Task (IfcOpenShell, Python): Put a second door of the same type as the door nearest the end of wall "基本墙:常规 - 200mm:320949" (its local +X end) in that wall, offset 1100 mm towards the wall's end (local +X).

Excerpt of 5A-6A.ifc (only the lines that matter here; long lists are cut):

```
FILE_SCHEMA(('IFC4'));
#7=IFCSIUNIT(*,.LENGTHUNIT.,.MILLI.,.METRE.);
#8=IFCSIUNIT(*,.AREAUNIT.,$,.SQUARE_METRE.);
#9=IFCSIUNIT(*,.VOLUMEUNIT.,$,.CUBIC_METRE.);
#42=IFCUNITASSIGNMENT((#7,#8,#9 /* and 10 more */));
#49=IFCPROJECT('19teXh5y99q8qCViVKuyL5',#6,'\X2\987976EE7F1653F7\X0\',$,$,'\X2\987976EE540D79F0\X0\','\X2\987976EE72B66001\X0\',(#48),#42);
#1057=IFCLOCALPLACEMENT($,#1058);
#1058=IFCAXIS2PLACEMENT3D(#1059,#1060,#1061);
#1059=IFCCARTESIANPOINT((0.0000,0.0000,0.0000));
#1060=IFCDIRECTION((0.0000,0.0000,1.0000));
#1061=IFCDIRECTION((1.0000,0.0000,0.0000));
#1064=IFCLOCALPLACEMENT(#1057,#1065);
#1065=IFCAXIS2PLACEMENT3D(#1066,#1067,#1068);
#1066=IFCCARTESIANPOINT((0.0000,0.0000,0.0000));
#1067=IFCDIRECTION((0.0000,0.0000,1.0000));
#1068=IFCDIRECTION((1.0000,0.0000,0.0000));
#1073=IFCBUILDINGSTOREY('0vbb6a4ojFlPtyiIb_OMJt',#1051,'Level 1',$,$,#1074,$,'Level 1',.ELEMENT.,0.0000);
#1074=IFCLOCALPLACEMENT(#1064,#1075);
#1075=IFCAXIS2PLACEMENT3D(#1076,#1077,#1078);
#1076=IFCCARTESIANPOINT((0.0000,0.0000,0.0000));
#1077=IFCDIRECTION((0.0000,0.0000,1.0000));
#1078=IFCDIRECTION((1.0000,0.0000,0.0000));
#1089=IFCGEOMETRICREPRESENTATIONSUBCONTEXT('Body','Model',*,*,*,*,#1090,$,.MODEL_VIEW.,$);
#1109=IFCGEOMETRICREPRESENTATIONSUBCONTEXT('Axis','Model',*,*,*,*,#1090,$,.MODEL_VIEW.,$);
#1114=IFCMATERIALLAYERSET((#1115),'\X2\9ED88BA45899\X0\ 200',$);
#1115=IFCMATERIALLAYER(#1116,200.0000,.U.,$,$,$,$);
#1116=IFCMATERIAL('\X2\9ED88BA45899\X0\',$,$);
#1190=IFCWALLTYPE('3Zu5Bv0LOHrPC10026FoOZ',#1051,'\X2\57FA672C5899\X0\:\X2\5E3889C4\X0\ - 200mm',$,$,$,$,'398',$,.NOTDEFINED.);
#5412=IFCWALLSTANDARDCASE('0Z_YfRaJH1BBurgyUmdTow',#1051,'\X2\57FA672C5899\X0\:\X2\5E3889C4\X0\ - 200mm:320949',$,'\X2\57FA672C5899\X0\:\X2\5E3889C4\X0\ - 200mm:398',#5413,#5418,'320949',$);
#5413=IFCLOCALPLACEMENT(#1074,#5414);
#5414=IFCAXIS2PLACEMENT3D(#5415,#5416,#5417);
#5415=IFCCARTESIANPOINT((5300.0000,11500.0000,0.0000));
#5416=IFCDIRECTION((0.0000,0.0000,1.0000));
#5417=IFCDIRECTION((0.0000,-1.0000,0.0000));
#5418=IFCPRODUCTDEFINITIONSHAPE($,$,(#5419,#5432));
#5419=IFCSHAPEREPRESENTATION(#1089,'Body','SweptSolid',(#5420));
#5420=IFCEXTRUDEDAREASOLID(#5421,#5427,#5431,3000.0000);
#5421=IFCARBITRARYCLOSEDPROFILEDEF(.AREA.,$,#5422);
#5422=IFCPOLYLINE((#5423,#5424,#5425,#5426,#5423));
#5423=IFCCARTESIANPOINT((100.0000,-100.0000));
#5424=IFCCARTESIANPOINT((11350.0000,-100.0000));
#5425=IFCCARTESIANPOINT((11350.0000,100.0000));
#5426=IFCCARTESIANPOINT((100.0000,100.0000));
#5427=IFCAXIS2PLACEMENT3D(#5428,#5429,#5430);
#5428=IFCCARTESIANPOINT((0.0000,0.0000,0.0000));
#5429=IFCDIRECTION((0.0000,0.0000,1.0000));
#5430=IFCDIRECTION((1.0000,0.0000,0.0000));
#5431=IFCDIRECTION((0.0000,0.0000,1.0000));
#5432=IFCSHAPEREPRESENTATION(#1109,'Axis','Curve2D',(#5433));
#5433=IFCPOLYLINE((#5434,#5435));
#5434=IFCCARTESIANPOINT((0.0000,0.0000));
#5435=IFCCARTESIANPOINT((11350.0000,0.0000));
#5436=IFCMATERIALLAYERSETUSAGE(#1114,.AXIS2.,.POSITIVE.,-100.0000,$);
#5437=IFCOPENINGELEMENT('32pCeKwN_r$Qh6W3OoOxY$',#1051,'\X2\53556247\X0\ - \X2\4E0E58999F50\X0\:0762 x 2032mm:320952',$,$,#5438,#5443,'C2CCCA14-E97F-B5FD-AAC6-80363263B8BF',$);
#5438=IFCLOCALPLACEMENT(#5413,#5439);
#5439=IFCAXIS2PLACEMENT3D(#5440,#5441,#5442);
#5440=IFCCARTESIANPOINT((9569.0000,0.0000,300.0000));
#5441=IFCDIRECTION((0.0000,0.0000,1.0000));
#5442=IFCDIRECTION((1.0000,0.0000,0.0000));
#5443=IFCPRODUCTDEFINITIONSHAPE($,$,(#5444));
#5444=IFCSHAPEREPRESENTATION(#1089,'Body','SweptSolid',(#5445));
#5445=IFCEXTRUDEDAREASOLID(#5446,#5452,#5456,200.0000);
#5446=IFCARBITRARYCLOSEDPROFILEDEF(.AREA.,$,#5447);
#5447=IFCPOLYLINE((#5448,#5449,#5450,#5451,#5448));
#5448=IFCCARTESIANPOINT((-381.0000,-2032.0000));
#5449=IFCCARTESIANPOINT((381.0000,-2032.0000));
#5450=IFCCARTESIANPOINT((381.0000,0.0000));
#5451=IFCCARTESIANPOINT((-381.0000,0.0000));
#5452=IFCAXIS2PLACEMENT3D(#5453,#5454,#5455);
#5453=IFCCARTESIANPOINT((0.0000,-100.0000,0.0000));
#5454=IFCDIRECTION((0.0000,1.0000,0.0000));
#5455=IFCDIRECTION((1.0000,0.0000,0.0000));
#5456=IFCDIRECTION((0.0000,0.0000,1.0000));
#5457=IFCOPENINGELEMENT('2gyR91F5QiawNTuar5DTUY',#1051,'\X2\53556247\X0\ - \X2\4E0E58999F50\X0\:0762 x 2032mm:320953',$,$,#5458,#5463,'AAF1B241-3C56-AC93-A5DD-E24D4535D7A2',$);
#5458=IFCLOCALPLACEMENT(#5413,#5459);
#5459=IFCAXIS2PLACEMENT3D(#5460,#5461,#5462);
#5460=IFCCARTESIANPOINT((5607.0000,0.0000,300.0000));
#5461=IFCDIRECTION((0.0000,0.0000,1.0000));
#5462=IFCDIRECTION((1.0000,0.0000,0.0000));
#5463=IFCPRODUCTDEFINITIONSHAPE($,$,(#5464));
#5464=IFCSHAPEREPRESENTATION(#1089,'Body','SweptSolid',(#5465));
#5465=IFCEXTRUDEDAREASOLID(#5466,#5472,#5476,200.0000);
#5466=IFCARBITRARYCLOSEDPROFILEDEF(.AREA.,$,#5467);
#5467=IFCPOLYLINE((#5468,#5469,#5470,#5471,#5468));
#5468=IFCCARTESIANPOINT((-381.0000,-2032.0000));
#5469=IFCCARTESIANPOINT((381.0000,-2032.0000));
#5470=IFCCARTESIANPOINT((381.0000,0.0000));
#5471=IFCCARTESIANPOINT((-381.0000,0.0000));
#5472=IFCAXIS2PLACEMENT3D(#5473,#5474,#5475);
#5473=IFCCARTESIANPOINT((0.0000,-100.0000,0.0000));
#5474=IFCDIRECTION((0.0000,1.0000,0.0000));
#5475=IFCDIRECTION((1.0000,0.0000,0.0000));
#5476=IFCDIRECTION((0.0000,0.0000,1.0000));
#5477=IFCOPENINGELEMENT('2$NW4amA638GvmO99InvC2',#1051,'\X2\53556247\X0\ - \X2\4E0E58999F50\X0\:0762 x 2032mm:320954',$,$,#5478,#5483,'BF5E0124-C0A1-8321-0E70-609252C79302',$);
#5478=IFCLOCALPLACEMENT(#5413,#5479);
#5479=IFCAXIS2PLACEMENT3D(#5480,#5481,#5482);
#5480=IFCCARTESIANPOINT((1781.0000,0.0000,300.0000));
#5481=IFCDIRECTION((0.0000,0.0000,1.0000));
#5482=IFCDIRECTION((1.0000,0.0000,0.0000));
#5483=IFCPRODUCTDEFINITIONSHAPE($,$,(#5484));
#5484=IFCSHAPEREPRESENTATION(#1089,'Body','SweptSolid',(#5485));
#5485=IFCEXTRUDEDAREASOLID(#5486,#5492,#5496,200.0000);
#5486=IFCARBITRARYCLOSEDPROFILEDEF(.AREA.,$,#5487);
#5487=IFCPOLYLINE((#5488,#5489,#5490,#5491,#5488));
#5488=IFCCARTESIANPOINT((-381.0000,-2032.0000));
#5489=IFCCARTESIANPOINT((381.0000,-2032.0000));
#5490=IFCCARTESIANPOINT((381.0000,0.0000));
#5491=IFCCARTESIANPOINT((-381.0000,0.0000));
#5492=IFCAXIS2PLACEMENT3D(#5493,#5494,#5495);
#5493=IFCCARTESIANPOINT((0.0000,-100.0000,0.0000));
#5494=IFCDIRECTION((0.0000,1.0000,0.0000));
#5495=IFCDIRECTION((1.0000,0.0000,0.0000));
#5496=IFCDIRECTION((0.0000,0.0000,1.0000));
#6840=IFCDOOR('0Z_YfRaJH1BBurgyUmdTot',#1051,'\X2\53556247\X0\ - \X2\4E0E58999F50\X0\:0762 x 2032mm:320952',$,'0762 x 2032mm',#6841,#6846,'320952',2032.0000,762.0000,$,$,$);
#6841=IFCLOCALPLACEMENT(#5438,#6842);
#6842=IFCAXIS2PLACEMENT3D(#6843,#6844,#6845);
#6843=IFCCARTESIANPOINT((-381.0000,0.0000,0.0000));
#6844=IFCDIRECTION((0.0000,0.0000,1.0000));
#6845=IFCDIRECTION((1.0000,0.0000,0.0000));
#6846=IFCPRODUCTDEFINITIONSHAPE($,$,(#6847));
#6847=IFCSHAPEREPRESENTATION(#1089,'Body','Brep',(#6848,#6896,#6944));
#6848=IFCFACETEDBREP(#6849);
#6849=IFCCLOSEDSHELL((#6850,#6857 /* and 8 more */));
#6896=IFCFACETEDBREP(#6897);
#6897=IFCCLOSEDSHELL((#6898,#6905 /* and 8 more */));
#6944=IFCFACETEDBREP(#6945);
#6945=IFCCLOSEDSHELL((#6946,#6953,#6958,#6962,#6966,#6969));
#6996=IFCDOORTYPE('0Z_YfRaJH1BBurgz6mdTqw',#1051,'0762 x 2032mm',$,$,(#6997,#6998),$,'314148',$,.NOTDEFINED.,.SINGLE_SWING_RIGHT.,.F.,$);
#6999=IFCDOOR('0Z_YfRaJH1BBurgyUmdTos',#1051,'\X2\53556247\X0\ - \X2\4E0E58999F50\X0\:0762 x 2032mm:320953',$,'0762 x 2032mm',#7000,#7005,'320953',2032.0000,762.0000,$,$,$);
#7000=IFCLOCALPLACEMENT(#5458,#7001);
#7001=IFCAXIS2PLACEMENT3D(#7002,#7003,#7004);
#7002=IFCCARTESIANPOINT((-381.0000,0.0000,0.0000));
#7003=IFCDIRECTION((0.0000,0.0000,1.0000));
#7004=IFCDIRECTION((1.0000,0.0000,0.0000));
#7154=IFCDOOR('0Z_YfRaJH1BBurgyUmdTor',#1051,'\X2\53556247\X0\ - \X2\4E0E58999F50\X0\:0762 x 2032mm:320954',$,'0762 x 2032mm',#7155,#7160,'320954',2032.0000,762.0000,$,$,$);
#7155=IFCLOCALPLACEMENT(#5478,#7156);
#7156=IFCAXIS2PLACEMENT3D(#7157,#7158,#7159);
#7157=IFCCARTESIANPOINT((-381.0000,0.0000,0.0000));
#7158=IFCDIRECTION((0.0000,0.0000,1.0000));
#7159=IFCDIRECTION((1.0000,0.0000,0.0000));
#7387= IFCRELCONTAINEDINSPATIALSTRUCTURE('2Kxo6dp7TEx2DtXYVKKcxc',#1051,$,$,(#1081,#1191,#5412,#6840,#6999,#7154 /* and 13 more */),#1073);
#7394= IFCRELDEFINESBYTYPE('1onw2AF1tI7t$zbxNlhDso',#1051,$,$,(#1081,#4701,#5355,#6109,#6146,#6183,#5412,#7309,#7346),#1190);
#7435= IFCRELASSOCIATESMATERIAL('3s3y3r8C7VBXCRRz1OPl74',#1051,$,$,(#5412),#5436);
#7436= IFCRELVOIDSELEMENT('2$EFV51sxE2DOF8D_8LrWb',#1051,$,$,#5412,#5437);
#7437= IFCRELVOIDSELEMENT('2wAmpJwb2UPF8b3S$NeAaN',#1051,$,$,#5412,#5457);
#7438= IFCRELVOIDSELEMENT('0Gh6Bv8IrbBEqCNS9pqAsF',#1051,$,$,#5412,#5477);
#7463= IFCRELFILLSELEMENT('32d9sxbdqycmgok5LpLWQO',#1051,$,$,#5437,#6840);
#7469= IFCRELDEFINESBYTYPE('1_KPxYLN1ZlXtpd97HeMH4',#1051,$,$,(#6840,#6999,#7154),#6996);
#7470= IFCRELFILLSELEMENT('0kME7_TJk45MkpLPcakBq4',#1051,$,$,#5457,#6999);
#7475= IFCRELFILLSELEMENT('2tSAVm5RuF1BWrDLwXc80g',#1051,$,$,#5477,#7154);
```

```python
import ifcopenshell
import ifcopenshell.api.feature
import ifcopenshell.api.geometry
import ifcopenshell.api.root
import ifcopenshell.geom
import ifcopenshell.util.element
import ifcopenshell.util.placement
import ifcopenshell.util.shape
import ifcopenshell.util.unit

model = ifcopenshell.open("5A-6A.ifc")
unit_scale = ifcopenshell.util.unit.calculate_unit_scale(model)
settings = ifcopenshell.geom.settings()


def volume(element):
    """Net volume in cubic metres, openings subtracted."""
    shape = ifcopenshell.geom.create_shape(settings, element)
    return ifcopenshell.util.shape.get_volume(shape.geometry)


def reuse_history(source, copy):
    """copy_class also copies each property set's owner history, people and application; keep the originals."""
    for rel in copy.IsDefinedBy:
        if rel.is_a("IfcRelDefinesByProperties") and (history := rel.RelatingPropertyDefinition.OwnerHistory):
            rel.RelatingPropertyDefinition.OwnerHistory = source.OwnerHistory
            ifcopenshell.util.element.remove_deep2(model, history)


door = model.by_id(6840)
opening = door.FillsVoids[0].RelatingOpeningElement
wall = opening.VoidsElements[0].RelatingBuildingElement
before = volume(wall)
shift = ifcopenshell.util.placement.get_local_placement(wall.ObjectPlacement)[:3, 0] * 1.1 / unit_scale

# copy_class copies the void relationship, type, container and properties, but no geometry.
new_opening = ifcopenshell.api.root.copy_class(model, product=opening)
new_opening.Representation = ifcopenshell.util.element.copy_deep(
    model, opening.Representation, exclude=["IfcGeometricRepresentationContext", "IfcRepresentationMap"]
)
new_opening.Name = "单扇 - 与墙齐:0762 x 2032mm"
new_opening.Tag = None
new_door = ifcopenshell.api.root.copy_class(model, product=door)
new_door.Representation = ifcopenshell.util.element.copy_deep(
    model, door.Representation, exclude=["IfcGeometricRepresentationContext", "IfcRepresentationMap"]
)
new_door.Name = "单扇 - 与墙齐:0762 x 2032mm"
new_door.Tag = None
reuse_history(door, new_door)
ifcopenshell.api.feature.add_filling(model, opening=new_opening, element=new_door)

for old, new in ((opening, new_opening), (door, new_door)):
    matrix = ifcopenshell.util.placement.get_local_placement(old.ObjectPlacement)
    matrix[:3, 3] += shift
    ifcopenshell.api.geometry.edit_object_placement(model, product=new, matrix=matrix, is_si=False)

after = volume(wall)

print(f"wall volume {before:.3f} -> {after:.3f} m3")

model.write("5A-6A_rev.ifc")
```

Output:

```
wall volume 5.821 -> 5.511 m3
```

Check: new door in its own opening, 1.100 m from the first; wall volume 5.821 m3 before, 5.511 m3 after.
